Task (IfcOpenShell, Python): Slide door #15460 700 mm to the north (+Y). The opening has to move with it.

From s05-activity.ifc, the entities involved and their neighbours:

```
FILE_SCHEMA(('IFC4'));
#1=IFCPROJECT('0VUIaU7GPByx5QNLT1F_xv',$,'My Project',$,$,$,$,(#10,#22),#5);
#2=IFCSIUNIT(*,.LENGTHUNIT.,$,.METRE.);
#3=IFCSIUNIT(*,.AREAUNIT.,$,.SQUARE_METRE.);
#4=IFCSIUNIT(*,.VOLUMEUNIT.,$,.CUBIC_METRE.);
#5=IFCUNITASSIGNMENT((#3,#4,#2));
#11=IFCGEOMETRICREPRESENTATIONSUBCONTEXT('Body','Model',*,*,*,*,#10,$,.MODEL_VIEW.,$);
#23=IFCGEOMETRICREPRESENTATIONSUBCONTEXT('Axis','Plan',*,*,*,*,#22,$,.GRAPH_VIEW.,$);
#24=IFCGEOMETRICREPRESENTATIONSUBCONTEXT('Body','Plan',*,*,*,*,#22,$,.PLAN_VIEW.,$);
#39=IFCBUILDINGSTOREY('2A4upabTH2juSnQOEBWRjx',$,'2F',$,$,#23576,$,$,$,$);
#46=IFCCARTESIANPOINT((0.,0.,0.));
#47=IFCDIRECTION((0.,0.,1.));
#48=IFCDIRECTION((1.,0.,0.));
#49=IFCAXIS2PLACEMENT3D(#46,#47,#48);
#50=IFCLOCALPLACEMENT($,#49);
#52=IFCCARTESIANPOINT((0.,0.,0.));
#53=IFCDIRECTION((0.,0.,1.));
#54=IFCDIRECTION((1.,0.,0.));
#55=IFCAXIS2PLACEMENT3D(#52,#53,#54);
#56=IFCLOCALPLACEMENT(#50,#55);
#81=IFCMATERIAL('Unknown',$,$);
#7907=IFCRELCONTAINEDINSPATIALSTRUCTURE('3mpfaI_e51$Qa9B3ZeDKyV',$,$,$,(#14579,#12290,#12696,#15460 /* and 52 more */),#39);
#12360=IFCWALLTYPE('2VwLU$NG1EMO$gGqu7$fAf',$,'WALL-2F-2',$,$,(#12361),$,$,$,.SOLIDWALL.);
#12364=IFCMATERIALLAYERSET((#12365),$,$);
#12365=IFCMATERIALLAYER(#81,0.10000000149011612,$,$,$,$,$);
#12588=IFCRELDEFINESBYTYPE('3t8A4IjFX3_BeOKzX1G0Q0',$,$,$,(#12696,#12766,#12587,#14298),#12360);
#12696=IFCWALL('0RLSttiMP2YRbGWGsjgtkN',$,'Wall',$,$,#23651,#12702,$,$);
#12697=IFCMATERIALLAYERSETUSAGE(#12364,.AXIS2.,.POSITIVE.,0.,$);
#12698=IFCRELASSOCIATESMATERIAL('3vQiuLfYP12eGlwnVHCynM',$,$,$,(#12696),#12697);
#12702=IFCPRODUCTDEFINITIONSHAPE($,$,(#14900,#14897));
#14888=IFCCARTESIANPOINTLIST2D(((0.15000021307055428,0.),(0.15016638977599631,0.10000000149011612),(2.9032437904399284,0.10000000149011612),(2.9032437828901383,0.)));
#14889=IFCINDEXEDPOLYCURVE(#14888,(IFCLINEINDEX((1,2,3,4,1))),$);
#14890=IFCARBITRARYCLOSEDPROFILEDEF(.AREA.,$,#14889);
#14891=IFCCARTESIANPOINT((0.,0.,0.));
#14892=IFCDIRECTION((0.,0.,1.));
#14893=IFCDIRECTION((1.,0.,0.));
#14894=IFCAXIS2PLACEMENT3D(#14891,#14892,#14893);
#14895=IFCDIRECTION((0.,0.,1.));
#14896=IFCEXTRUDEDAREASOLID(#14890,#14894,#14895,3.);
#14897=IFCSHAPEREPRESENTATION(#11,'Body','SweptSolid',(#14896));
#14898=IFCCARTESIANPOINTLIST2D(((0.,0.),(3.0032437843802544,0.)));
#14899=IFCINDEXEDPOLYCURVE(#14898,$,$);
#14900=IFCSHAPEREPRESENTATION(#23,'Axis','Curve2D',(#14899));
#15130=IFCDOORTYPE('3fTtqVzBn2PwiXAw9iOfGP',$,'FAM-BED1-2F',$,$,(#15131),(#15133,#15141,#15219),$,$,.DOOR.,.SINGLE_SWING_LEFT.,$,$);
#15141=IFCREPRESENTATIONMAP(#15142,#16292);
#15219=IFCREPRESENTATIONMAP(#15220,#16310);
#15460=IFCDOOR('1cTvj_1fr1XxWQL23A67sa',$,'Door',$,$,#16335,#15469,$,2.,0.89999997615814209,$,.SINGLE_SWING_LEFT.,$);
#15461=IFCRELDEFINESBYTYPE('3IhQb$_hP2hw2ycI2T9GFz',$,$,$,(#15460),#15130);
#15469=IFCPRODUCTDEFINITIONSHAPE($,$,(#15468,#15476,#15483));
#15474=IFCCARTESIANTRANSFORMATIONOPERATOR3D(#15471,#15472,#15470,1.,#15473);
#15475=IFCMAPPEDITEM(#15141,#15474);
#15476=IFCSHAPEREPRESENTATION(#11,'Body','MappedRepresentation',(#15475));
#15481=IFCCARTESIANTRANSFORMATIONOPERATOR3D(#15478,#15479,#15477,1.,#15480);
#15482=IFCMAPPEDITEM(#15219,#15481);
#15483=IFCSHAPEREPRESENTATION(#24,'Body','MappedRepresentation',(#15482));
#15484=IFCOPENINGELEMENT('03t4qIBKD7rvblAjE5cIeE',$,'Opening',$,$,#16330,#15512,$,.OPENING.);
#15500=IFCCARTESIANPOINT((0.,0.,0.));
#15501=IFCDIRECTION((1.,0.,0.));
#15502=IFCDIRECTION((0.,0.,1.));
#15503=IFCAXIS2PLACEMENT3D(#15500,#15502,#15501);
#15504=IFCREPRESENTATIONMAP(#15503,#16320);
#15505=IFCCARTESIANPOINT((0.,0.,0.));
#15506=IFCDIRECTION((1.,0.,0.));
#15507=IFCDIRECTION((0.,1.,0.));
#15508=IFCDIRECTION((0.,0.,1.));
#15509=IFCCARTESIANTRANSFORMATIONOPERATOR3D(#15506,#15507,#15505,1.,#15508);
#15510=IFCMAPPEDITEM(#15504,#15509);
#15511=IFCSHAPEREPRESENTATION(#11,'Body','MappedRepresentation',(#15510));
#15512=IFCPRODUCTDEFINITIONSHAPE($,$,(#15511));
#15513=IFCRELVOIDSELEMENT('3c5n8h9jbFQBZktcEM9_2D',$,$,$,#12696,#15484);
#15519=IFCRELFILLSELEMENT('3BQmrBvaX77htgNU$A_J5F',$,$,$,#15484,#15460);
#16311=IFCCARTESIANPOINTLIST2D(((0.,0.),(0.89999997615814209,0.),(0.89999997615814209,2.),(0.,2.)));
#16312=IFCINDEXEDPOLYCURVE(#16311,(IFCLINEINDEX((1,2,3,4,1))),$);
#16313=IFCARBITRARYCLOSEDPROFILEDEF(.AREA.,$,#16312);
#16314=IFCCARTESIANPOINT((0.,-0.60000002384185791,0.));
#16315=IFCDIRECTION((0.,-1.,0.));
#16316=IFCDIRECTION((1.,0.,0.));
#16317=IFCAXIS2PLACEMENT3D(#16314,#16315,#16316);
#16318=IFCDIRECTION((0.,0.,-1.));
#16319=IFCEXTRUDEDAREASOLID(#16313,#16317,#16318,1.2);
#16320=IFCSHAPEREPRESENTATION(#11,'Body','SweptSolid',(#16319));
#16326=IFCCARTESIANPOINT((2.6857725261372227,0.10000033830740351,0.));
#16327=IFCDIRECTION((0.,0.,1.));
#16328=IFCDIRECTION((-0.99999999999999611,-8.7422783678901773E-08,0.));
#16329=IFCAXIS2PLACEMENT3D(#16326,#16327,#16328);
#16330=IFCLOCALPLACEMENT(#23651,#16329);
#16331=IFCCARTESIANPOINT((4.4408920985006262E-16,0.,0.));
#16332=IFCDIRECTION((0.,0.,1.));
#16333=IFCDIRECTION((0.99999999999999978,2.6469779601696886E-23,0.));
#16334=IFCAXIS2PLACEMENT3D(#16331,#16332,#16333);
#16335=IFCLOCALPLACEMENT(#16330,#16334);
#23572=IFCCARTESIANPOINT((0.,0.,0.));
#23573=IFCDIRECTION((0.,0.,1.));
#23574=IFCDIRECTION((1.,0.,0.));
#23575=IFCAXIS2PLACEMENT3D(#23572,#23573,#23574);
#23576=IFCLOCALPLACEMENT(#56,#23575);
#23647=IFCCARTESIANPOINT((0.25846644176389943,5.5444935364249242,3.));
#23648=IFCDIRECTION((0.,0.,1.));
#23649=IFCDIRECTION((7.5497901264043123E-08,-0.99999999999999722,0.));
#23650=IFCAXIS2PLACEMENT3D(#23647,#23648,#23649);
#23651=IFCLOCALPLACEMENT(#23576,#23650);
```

```python
import ifcopenshell
import ifcopenshell.api.geometry
import ifcopenshell.util.placement
import ifcopenshell.util.unit

model = ifcopenshell.open("s05-activity.ifc")
unit_scale = ifcopenshell.util.unit.calculate_unit_scale(model)

door = model.by_guid("1cTvj_1fr1XxWQL23A67sa")
opening = door.FillsVoids[0].RelatingOpeningElement
wall = opening.VoidsElements[0].RelatingBuildingElement

wall_matrix = ifcopenshell.util.placement.get_local_placement(wall.ObjectPlacement)
shift = wall_matrix[:3, 0] * -0.7 / unit_scale
before = ifcopenshell.util.placement.get_local_placement(door.ObjectPlacement)[:3, 3].copy()

# The door is placed relative to its opening, so it follows when the opening moves.
matrix = ifcopenshell.util.placement.get_local_placement(opening.ObjectPlacement)
matrix[:3, 3] += shift
ifcopenshell.api.geometry.edit_object_placement(
    model, product=opening, matrix=matrix, is_si=False, should_transform_children=True
)

after = ifcopenshell.util.placement.get_local_placement(door.ObjectPlacement)[:3, 3]
print("door moved by", (after - before).round(3) + 0.0)

model.write("s05-activity_v2.ifc")
```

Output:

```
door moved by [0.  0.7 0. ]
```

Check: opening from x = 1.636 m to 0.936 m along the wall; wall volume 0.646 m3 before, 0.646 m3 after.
